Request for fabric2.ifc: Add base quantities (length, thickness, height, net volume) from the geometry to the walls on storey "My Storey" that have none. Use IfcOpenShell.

First a look at what the model holds.

```python
import ifcopenshell
import ifcopenshell.util.element
import ifcopenshell.util.unit

model = ifcopenshell.open("fabric2.ifc")
print(model.schema)
for unit_type in ("LENGTHUNIT", "AREAUNIT", "VOLUMEUNIT"):
    print(unit_type, ifcopenshell.util.unit.calculate_unit_scale(model, unit_type))
storey = next(s for s in model.by_type("IfcBuildingStorey") if s.Name == "My Storey")
walls = [e for e in ifcopenshell.util.element.get_decomposition(storey) if e.is_a("IfcWall")]
for e in sorted(walls, key=lambda e: e.id()):
    print(e.id(), e.is_a(), e.Name, list(ifcopenshell.util.element.get_psets(e, qtos_only=True)), sep=" | ")
```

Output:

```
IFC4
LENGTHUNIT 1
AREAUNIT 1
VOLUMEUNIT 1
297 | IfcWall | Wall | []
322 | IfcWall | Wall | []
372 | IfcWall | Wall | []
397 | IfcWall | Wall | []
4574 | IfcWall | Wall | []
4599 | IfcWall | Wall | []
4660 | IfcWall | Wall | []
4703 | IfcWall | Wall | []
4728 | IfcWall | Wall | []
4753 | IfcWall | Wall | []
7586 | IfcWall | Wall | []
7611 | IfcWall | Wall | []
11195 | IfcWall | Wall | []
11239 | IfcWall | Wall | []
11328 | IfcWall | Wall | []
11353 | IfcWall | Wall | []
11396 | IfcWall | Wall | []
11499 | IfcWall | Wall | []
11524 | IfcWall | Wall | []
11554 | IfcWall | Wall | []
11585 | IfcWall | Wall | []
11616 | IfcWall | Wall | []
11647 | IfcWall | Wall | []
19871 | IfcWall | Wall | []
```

```python
import ifcopenshell
import ifcopenshell.api.pset
import ifcopenshell.geom
import ifcopenshell.util.element
import ifcopenshell.util.shape
import ifcopenshell.util.unit

model = ifcopenshell.open("fabric2.ifc")
unit_scale = ifcopenshell.util.unit.calculate_unit_scale(model)
volume_scale = ifcopenshell.util.unit.calculate_unit_scale(model, "VOLUMEUNIT")
settings = ifcopenshell.geom.settings()

storey = next(s for s in model.by_type("IfcBuildingStorey") if s.Name == "My Storey")
walls = [e for e in ifcopenshell.util.element.get_decomposition(storey) if e.is_a("IfcWall")]

for e in sorted(walls, key=lambda e: e.id()):
    if ifcopenshell.util.element.get_psets(e, qtos_only=True, should_inherit=False):
        continue
    # Geometry comes back in metres, in the element's own axes.
    shape = ifcopenshell.geom.create_shape(settings, e)
    values = {
        "Length": ifcopenshell.util.shape.get_x(shape.geometry) / unit_scale,
        "Width": ifcopenshell.util.shape.get_y(shape.geometry) / unit_scale,
        "Height": ifcopenshell.util.shape.get_z(shape.geometry) / unit_scale,
        "NetVolume": ifcopenshell.util.shape.get_volume(shape.geometry) / volume_scale,
    }
    qto = ifcopenshell.api.pset.add_qto(model, product=e, name="Qto_WallBaseQuantities")
    ifcopenshell.api.pset.edit_qto(model, qto=qto, properties=values)
    print(e.id(), {k: round(v, 3) for k, v in values.items()})

model.write("fabric2_edited.ifc")
```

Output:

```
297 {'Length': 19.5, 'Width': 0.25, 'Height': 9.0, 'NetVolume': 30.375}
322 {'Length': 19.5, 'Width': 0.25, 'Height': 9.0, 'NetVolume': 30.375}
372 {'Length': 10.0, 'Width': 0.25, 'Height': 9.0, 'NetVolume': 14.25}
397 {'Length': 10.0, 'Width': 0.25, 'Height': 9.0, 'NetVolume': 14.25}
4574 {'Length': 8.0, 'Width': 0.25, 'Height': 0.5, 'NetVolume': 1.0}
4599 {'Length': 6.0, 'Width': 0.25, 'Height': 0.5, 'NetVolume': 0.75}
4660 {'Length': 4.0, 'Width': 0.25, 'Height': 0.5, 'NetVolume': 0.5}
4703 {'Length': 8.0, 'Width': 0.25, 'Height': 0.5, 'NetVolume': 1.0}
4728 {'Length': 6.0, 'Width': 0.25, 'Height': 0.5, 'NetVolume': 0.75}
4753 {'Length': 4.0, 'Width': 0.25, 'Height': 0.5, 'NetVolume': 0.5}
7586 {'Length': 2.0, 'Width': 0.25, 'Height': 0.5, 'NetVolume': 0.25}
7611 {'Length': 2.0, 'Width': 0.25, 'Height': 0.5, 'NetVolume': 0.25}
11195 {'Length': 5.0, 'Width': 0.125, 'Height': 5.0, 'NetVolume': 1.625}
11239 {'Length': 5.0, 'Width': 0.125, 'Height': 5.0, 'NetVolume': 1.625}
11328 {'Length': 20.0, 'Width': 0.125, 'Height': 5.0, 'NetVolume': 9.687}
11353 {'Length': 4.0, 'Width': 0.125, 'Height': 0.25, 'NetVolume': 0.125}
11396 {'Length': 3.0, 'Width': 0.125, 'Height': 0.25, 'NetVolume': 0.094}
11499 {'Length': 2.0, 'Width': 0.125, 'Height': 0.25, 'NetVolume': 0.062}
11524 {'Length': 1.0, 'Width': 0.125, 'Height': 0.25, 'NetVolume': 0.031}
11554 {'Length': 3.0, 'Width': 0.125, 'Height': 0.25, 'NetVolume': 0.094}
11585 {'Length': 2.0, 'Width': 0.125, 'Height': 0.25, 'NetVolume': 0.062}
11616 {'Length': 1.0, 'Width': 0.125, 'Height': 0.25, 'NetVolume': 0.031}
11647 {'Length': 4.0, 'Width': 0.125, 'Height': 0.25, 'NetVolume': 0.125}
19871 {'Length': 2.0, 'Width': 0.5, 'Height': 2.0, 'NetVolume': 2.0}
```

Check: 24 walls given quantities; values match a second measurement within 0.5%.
